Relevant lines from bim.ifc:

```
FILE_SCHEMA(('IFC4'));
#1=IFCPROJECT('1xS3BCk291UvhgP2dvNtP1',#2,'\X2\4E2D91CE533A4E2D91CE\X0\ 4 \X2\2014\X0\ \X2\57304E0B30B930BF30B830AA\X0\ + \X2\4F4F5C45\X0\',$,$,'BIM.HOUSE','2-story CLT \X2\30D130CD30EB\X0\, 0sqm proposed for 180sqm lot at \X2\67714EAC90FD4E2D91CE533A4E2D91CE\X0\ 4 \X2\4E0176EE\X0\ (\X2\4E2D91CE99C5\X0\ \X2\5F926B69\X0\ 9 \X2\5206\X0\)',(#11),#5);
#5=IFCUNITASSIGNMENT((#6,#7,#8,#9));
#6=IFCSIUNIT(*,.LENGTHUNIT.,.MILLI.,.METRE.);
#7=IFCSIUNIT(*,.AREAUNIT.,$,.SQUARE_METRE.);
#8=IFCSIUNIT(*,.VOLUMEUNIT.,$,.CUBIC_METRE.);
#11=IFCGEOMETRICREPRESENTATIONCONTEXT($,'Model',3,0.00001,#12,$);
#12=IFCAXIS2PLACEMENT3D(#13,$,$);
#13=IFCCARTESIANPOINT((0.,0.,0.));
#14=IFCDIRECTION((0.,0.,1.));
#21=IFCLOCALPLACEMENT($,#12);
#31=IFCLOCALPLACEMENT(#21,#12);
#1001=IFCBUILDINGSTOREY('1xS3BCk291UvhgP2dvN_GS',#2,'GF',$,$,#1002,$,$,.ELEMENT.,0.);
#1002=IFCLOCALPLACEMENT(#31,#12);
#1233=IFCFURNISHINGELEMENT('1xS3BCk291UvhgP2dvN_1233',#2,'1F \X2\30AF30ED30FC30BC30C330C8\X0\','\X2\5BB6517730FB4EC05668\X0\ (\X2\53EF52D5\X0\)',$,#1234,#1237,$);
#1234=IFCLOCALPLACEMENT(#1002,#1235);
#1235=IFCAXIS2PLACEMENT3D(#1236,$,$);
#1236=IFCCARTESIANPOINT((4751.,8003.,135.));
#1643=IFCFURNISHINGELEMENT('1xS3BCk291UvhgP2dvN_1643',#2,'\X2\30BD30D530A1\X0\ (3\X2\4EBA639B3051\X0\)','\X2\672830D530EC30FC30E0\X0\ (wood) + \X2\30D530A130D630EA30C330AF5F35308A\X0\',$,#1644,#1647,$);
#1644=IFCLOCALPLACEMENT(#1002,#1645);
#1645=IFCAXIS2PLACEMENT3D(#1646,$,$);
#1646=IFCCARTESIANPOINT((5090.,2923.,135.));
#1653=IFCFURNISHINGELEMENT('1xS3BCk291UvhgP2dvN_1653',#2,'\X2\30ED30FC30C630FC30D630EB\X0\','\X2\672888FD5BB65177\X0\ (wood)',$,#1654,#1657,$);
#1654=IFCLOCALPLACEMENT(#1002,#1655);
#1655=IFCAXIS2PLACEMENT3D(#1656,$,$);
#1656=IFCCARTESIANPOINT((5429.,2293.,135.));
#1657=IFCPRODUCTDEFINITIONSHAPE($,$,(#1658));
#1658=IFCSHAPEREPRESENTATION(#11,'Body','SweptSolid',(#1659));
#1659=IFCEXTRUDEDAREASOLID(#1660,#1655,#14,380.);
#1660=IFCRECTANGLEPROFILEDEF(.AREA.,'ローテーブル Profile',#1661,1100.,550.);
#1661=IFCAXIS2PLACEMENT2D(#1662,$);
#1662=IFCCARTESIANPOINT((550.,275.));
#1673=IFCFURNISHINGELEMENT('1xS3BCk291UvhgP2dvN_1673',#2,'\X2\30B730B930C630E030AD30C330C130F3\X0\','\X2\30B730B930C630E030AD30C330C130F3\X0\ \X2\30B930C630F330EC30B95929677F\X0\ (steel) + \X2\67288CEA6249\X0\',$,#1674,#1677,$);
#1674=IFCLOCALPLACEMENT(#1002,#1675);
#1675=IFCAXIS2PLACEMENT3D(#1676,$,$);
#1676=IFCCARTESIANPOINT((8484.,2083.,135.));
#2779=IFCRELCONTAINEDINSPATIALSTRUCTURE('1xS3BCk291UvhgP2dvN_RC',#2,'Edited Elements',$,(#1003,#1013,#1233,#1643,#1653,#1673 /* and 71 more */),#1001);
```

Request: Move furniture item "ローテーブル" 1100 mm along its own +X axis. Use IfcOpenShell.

```python
import ifcopenshell
import ifcopenshell.api.geometry
import ifcopenshell.util.placement

model = ifcopenshell.open("bim.ifc")

item = model.by_id(1653)
matrix = ifcopenshell.util.placement.get_local_placement(item.ObjectPlacement)
matrix[:3, 3] += matrix[:3, 0] * 1100.0
ifcopenshell.api.geometry.edit_object_placement(model, product=item, matrix=matrix, is_si=False)

print(ifcopenshell.util.placement.get_local_placement(item.ObjectPlacement).round(3) + 0.0)

model.write("bim-out.ifc")
```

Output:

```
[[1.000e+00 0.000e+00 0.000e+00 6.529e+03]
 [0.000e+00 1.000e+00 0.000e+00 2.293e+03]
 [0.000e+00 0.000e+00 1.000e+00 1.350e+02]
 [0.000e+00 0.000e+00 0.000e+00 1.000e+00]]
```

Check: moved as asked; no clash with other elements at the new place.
